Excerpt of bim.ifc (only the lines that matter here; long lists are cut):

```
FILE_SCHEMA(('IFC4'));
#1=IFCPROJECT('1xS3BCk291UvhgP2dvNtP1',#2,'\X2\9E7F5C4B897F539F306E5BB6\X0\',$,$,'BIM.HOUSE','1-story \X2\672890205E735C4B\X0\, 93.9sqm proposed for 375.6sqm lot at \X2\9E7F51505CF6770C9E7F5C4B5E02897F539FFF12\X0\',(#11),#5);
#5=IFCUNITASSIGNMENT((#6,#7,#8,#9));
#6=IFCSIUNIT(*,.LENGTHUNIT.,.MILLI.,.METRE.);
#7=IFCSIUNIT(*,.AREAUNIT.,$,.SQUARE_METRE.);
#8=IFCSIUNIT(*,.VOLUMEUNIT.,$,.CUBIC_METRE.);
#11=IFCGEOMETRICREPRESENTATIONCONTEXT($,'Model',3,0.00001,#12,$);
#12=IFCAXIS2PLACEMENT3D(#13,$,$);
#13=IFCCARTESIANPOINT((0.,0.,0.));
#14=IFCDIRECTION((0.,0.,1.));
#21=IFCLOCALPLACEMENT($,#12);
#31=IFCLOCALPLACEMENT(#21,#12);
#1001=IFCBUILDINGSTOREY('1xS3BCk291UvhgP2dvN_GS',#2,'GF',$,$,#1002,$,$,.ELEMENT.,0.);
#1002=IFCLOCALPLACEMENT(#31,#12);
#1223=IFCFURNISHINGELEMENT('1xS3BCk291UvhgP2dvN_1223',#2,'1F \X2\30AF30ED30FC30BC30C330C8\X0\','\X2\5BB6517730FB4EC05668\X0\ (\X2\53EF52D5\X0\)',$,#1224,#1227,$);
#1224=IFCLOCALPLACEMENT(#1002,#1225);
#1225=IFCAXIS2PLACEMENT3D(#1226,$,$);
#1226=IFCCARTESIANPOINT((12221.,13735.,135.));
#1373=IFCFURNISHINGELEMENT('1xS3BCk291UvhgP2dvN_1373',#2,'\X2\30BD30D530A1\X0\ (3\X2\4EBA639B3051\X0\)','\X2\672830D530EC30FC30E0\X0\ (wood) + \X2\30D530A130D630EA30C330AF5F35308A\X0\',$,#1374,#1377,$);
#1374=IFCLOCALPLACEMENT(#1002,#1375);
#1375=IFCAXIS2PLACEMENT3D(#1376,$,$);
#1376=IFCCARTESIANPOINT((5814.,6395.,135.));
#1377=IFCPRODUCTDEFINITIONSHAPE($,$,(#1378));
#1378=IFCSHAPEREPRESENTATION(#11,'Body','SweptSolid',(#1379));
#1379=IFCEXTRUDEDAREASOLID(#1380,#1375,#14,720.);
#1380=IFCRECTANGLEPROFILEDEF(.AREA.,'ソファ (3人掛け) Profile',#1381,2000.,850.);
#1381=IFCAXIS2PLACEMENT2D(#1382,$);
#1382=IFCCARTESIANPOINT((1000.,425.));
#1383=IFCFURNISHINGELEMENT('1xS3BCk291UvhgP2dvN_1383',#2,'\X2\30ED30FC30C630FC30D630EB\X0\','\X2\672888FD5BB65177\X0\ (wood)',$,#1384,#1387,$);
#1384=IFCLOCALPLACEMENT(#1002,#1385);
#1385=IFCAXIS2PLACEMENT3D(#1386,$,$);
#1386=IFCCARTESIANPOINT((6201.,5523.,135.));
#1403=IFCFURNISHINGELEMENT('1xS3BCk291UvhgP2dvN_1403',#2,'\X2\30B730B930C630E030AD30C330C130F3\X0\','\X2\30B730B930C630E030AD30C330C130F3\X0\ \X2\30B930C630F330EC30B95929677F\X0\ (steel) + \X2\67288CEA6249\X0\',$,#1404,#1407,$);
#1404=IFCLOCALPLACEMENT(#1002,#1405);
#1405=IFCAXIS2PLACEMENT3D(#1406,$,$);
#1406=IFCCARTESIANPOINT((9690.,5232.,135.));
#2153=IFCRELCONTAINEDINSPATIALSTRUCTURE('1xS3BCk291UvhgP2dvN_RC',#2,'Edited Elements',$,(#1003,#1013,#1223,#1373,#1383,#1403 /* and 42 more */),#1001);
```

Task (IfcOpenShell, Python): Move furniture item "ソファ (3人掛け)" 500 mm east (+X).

```python
import ifcopenshell
import ifcopenshell.api.geometry
import ifcopenshell.util.placement
import ifcopenshell.util.unit

model = ifcopenshell.open("bim.ifc")
unit_scale = ifcopenshell.util.unit.calculate_unit_scale(model)

item = model.by_guid("1xS3BCk291UvhgP2dvN_1373")
matrix = ifcopenshell.util.placement.get_local_placement(item.ObjectPlacement)
matrix[0, 3] += 0.5 / unit_scale
ifcopenshell.api.geometry.edit_object_placement(model, product=item, matrix=matrix, is_si=False)

print(ifcopenshell.util.placement.get_local_placement(item.ObjectPlacement).round(3) + 0.0)

model.write("bim-out.ifc")
```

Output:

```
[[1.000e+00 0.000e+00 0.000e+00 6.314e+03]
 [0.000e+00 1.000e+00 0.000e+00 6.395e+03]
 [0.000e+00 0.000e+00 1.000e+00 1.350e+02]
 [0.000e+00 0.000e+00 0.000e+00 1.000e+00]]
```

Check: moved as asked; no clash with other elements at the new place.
